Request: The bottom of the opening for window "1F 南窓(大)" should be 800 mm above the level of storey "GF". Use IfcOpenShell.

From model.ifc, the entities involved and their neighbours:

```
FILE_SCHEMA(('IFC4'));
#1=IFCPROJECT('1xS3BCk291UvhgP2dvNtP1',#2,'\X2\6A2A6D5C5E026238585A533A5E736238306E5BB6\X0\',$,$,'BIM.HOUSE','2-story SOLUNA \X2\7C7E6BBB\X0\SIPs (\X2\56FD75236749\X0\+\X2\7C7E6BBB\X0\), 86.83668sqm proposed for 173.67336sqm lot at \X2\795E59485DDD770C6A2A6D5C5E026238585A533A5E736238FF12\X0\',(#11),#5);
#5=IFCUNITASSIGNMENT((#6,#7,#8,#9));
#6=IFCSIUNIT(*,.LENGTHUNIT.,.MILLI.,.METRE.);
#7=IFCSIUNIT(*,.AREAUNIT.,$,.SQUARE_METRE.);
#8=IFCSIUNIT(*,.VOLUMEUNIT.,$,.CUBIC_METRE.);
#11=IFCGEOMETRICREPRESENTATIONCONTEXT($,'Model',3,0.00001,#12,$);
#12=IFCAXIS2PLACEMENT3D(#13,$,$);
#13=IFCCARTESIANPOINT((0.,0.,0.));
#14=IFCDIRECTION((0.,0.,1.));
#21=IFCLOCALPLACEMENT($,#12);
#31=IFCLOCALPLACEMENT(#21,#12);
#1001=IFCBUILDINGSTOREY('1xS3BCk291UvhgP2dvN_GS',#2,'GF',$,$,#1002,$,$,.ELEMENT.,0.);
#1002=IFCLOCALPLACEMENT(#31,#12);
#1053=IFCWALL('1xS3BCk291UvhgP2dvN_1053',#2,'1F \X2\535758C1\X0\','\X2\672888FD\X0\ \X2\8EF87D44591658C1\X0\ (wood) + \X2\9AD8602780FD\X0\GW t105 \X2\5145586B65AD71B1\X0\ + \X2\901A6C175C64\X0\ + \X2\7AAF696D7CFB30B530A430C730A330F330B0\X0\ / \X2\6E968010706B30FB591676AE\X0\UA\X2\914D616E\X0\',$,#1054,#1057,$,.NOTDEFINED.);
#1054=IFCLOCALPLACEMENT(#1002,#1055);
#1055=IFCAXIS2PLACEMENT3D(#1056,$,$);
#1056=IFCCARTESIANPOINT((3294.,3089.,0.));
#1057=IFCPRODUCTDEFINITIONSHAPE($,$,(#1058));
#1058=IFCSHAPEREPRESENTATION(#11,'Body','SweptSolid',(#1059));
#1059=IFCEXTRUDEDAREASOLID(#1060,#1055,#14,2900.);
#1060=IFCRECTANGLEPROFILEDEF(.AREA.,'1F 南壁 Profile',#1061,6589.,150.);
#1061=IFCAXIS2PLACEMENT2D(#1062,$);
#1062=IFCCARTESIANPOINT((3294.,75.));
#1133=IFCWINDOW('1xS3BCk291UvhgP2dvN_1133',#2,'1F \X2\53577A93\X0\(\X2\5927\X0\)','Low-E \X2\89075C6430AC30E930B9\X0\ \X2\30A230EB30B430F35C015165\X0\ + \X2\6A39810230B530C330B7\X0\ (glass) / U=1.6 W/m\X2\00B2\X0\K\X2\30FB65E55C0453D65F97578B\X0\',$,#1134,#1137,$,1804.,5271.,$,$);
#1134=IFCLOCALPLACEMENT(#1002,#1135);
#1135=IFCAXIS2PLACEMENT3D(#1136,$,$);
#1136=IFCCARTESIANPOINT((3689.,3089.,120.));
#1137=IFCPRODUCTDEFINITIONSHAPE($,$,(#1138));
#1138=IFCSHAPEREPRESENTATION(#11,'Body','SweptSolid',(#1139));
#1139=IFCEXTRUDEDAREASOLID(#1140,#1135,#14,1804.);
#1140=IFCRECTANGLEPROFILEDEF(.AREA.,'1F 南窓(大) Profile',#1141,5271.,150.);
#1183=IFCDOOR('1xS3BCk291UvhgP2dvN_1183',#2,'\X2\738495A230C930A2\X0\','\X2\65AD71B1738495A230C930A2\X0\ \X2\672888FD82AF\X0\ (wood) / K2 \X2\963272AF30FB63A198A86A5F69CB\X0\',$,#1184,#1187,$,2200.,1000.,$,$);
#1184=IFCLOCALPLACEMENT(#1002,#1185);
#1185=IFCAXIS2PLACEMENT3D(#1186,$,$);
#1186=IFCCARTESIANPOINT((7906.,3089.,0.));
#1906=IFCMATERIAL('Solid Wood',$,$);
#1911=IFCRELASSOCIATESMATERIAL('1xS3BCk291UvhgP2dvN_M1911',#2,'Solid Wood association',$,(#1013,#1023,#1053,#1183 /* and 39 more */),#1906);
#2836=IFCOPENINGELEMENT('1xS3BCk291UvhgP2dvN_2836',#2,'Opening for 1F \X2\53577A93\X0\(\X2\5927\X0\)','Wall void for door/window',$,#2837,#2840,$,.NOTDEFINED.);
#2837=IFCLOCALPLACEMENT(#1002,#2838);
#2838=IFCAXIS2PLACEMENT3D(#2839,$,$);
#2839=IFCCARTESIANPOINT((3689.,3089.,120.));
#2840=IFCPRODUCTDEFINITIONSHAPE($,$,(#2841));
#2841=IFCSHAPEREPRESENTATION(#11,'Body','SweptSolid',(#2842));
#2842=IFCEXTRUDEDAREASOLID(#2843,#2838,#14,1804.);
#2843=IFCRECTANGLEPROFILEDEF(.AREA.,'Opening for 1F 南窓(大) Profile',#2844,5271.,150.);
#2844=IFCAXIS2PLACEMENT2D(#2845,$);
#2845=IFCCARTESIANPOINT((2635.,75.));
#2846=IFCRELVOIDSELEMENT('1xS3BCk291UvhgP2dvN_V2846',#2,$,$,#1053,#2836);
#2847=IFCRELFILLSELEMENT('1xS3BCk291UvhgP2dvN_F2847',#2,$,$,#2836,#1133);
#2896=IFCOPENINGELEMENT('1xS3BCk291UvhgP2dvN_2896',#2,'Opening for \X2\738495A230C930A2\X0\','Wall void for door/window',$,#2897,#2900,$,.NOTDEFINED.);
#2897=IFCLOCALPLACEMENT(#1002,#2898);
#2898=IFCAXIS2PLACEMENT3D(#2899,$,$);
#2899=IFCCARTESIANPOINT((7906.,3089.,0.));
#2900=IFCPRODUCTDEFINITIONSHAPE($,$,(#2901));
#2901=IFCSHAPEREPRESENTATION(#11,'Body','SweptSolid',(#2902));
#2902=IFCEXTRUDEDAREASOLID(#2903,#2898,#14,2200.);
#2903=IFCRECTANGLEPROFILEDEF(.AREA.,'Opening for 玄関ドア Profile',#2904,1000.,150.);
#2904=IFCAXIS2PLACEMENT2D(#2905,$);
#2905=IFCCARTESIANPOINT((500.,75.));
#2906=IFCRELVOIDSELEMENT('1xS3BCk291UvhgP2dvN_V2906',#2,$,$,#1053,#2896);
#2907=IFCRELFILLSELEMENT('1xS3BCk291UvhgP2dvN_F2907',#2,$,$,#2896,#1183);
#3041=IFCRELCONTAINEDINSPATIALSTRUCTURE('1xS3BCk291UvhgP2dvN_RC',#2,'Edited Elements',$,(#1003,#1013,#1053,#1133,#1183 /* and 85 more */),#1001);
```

```python
import numpy as np
import ifcopenshell
import ifcopenshell.api.geometry
import ifcopenshell.geom
import ifcopenshell.util.element
import ifcopenshell.util.placement
import ifcopenshell.util.shape
import ifcopenshell.util.unit

model = ifcopenshell.open("model.ifc")
unit_scale = ifcopenshell.util.unit.calculate_unit_scale(model)

window = model.by_guid("1xS3BCk291UvhgP2dvN_1133")
opening = window.FillsVoids[0].RelatingOpeningElement
storey = ifcopenshell.util.element.get_container(window, ifc_class="IfcBuildingStorey")
level = ifcopenshell.util.placement.get_local_placement(storey.ObjectPlacement)[2, 3]

# The opening's origin need not be at the sill, so measure its lowest point.
shape = ifcopenshell.geom.create_shape(ifcopenshell.geom.settings(), opening)
bottom = ifcopenshell.util.shape.get_shape_bottom_elevation(shape, shape.geometry) / unit_scale
dz = level + 0.8 / unit_scale - bottom

shift = np.array([0.0, 0.0, dz])
# The window is not placed relative to its opening, so move both.
for product in (opening, window):
    matrix = ifcopenshell.util.placement.get_local_placement(product.ObjectPlacement)
    matrix[:3, 3] += shift
    ifcopenshell.api.geometry.edit_object_placement(model, product=product, matrix=matrix, is_si=False)

print(f"moved by {dz * unit_scale:+.3f} m")

model.write("model_v2.ifc")
```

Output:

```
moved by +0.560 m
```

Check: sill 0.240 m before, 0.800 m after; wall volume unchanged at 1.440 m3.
